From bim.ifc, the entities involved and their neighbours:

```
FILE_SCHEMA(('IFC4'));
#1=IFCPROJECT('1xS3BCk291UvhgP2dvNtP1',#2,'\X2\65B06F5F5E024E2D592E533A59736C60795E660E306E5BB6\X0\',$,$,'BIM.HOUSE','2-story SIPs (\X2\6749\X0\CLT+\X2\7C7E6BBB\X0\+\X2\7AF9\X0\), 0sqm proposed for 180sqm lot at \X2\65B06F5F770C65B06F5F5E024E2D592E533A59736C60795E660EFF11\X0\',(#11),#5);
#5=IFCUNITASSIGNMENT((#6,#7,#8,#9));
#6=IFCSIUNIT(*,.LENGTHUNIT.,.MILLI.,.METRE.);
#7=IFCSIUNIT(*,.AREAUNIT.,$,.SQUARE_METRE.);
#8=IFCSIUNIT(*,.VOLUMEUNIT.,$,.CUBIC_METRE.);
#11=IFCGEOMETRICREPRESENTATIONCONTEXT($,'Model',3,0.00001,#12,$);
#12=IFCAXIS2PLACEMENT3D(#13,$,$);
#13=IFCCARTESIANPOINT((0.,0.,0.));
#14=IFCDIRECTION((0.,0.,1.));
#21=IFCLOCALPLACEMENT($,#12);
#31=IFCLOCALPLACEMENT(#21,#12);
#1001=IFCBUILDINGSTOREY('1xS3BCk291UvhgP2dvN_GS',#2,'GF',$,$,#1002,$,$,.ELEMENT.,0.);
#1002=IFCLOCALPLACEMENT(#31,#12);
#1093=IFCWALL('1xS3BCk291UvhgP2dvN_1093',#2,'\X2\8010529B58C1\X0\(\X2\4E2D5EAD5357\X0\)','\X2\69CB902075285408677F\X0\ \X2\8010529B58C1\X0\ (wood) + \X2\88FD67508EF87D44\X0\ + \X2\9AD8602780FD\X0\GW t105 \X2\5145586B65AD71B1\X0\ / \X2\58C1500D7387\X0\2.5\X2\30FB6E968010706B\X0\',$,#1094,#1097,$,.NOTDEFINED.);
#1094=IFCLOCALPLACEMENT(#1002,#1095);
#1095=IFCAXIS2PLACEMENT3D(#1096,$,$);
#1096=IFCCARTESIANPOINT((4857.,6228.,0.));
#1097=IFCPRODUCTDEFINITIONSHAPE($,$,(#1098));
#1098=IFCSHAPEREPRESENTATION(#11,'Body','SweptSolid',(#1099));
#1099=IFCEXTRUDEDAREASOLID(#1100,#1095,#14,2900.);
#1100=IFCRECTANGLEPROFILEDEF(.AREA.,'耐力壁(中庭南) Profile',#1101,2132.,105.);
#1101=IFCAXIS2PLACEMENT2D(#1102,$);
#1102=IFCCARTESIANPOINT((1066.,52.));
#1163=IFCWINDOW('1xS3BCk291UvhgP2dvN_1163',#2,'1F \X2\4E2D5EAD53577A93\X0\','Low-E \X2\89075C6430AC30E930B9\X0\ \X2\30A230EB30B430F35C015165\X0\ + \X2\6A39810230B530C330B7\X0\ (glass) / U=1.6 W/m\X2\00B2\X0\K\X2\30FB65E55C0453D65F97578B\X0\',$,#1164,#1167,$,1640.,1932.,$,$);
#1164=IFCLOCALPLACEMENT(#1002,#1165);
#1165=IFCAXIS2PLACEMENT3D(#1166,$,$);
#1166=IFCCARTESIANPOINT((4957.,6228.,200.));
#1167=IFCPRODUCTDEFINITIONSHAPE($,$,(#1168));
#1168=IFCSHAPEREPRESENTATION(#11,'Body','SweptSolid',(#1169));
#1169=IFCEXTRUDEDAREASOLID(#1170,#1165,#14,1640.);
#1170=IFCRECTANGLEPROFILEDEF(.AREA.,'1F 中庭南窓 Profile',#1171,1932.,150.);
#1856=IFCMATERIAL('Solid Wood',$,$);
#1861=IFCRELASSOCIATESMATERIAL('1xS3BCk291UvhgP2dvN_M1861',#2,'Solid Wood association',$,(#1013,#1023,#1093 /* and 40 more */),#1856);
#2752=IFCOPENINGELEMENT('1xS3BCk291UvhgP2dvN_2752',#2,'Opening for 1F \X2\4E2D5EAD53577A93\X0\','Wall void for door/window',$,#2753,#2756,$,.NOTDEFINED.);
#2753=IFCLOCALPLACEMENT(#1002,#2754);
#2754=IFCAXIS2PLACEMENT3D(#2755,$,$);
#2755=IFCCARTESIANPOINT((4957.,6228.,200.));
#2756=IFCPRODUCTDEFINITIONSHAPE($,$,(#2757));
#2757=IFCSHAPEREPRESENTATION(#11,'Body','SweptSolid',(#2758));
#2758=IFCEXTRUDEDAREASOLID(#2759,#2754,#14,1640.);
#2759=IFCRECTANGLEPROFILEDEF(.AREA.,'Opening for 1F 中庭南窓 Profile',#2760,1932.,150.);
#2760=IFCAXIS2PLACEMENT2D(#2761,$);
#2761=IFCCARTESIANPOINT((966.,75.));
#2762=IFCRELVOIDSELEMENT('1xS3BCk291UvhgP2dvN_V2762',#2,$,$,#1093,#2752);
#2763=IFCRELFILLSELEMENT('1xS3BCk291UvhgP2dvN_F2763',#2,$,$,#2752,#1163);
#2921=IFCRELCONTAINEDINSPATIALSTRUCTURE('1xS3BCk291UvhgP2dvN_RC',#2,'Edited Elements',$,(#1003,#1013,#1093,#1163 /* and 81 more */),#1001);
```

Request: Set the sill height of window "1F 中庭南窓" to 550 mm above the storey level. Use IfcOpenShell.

```python
import numpy as np
import ifcopenshell
import ifcopenshell.api.geometry
import ifcopenshell.geom
import ifcopenshell.util.element
import ifcopenshell.util.placement
import ifcopenshell.util.shape
import ifcopenshell.util.unit

model = ifcopenshell.open("bim.ifc")
unit_scale = ifcopenshell.util.unit.calculate_unit_scale(model)

window = model.by_id(1163)
opening = window.FillsVoids[0].RelatingOpeningElement
storey = ifcopenshell.util.element.get_container(window, ifc_class="IfcBuildingStorey")
level = ifcopenshell.util.placement.get_local_placement(storey.ObjectPlacement)[2, 3]

# The opening's origin need not be at the sill, so measure its lowest point.
shape = ifcopenshell.geom.create_shape(ifcopenshell.geom.settings(), opening)
bottom = ifcopenshell.util.shape.get_shape_bottom_elevation(shape, shape.geometry) / unit_scale
dz = level + 550.0 - bottom

shift = np.array([0.0, 0.0, dz])
# The window is not placed relative to its opening, so move both.
for product in (opening, window):
    matrix = ifcopenshell.util.placement.get_local_placement(product.ObjectPlacement)
    matrix[:3, 3] += shift
    ifcopenshell.api.geometry.edit_object_placement(model, product=product, matrix=matrix, is_si=False)

print(f"moved by {dz * unit_scale:+.3f} m")

model.write("bim_v2.ifc")
```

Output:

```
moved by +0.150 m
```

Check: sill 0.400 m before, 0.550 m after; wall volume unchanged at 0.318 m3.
